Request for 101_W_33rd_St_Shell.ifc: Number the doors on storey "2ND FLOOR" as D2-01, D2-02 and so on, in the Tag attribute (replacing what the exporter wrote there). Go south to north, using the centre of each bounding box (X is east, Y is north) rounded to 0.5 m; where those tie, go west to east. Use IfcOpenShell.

First a look at what the model holds.

```python
import ifcopenshell
import ifcopenshell.util.element
import ifcopenshell.util.placement

model = ifcopenshell.open("101_W_33rd_St_Shell.ifc")
print(model.schema)
storey = next(s for s in model.by_type("IfcBuildingStorey") if s.Name == "2ND FLOOR")
doors = [e for e in ifcopenshell.util.element.get_decomposition(storey) if e.is_a("IfcDoor")]
for e in sorted(doors, key=lambda e: e.id()):
    origin = ifcopenshell.util.placement.get_local_placement(e.ObjectPlacement)[:3, 3]
    print(e.id(), e.Tag, e.Name, origin.round(2) + 0.0, sep=" | ")
```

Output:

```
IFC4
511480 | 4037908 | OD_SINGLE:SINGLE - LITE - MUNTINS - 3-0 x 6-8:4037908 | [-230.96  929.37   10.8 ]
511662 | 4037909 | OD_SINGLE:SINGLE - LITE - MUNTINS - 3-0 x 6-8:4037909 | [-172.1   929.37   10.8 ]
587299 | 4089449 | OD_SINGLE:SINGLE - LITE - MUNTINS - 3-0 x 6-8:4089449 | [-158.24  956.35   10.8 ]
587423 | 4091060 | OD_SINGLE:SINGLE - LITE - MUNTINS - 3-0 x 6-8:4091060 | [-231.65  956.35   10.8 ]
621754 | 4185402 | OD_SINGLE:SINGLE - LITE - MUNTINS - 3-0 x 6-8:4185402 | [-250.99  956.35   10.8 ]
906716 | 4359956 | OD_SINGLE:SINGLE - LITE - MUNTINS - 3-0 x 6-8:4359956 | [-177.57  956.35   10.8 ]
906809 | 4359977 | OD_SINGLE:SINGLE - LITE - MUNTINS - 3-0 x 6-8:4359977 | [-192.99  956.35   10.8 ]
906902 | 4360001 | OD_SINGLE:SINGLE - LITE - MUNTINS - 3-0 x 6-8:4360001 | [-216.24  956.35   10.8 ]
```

```python
import ifcopenshell
import ifcopenshell.geom
import ifcopenshell.util.element
import ifcopenshell.util.shape

model = ifcopenshell.open("101_W_33rd_St_Shell.ifc")
settings = ifcopenshell.geom.settings()
settings.set("use-world-coords", True)


def centre(element):
    shape = ifcopenshell.geom.create_shape(settings, element)
    return ifcopenshell.util.shape.get_bbox_centroid(shape.geometry)


storey = next(s for s in model.by_type("IfcBuildingStorey") if s.Name == "2ND FLOOR")
doors = [e for e in ifcopenshell.util.element.get_decomposition(storey) if e.is_a("IfcDoor")]

# Insertion points can sit at a corner or the storey origin, so sort by the geometry (in metres).
centres = {e: centre(e) for e in doors}
doors.sort(key=lambda e: (round(centres[e][1] / 0.5), centres[e][0]))

for i, e in enumerate(doors, start=1):
    number = f"D2-{i:02d}"
    e.Tag = number
    print(e.id(), number)

model.write("101_W_33rd_St_Shell_edited.ifc")
```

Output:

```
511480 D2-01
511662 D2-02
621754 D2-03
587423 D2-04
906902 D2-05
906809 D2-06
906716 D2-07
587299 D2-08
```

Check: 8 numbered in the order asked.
